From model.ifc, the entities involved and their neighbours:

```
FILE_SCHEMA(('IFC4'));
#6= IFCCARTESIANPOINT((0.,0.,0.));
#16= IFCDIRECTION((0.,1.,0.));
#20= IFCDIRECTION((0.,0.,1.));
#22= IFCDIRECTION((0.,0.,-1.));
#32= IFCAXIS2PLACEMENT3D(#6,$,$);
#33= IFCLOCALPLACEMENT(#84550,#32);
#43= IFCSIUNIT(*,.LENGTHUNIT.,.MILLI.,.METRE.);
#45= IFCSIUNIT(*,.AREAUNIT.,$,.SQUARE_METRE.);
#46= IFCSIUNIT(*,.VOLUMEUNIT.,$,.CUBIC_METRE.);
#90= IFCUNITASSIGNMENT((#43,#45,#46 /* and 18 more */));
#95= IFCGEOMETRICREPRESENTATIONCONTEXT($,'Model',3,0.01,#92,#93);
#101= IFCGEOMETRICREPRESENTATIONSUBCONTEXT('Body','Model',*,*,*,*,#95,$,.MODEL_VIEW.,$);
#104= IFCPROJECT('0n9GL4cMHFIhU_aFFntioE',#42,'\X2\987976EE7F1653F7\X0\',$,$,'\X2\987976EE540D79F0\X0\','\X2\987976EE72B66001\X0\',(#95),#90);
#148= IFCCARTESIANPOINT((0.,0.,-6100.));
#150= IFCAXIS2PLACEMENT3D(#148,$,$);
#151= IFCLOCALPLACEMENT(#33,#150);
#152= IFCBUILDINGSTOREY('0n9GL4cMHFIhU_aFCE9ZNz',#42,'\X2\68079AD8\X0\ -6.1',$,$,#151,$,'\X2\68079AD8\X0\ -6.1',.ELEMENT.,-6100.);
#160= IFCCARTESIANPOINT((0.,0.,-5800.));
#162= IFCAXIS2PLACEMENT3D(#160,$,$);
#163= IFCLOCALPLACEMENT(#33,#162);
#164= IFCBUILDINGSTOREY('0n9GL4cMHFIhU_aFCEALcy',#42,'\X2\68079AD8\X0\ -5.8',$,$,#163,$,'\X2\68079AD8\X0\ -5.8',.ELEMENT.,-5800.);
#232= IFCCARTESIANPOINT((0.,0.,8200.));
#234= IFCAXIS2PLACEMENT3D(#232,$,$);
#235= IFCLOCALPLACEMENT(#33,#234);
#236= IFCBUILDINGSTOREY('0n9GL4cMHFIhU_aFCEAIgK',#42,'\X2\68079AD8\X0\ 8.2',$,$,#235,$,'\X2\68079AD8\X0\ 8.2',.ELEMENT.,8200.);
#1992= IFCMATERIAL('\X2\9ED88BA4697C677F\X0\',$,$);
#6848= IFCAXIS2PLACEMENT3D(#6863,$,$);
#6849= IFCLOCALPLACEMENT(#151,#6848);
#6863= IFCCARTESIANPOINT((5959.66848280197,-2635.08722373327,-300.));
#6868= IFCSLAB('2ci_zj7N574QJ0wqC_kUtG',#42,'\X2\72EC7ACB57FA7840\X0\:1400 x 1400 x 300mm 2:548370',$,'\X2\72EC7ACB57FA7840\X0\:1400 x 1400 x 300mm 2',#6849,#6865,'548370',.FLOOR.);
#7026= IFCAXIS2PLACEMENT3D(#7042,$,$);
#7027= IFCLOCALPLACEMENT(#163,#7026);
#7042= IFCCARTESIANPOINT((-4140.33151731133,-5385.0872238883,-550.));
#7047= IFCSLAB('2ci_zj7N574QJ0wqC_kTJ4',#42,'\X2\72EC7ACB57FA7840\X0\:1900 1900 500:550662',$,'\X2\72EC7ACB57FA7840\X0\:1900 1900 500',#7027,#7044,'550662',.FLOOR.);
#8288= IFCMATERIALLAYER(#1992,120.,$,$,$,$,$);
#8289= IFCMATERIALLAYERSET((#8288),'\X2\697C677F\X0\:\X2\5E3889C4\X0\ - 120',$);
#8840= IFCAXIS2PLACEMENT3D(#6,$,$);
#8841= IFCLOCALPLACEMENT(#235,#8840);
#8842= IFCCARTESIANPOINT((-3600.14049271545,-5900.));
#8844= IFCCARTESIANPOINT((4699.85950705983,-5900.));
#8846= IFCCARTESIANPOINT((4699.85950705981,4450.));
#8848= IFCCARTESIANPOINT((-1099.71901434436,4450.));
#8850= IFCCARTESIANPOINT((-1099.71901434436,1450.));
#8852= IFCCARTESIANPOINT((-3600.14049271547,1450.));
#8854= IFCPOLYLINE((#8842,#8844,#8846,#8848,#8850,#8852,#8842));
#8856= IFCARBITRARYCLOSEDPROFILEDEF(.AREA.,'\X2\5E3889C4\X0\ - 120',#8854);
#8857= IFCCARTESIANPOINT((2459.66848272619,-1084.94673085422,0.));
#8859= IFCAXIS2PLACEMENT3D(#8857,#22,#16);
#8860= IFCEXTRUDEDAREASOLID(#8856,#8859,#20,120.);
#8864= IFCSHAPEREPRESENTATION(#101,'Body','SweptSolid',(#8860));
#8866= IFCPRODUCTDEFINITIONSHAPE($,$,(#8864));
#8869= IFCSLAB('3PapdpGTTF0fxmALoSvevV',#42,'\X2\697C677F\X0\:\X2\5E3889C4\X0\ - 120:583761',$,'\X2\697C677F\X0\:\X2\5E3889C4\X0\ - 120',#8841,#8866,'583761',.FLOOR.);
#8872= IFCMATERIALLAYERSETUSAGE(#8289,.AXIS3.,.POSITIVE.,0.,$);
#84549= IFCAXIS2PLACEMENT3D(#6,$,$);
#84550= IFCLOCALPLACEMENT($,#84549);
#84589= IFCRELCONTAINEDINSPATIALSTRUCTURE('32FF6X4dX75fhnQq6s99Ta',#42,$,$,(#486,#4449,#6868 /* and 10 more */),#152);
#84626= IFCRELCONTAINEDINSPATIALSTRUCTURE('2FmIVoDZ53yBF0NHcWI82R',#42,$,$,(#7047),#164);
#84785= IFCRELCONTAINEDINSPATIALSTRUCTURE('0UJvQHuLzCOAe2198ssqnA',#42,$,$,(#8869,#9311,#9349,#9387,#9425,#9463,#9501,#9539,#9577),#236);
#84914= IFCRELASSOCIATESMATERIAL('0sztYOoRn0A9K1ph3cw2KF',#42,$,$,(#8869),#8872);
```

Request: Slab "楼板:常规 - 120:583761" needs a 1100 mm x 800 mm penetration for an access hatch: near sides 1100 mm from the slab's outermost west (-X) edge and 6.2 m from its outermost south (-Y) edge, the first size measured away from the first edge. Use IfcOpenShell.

```python
import numpy as np
import ifcopenshell
import ifcopenshell.api.feature
import ifcopenshell.api.geometry
import ifcopenshell.api.root
import ifcopenshell.geom
import ifcopenshell.util.placement
import ifcopenshell.util.representation
import ifcopenshell.util.shape
import ifcopenshell.util.unit

model = ifcopenshell.open("model.ifc")
unit_scale = ifcopenshell.util.unit.calculate_unit_scale(model)
settings = ifcopenshell.geom.settings()


def volume(element):
    """Net volume in cubic metres, openings subtracted."""
    shape = ifcopenshell.geom.create_shape(settings, element)
    return ifcopenshell.util.shape.get_volume(shape.geometry)


slab = model.by_guid("3PapdpGTTF0fxmALoSvevV")
before = volume(slab)

# Extent in the slab's own axes, in metres. The edges named are its -X and -Y sides.
slab_shape = ifcopenshell.geom.create_shape(settings, slab)
vertices = ifcopenshell.util.shape.get_vertices(slab_shape.geometry)
x_min, y_min, bottom = vertices.min(axis=0)
top = vertices[:, 2].max()

opening = ifcopenshell.api.root.create_entity(model, ifc_class="IfcOpeningElement", name="Access hatch opening", predefined_type="OPENING")
context = ifcopenshell.util.representation.get_context(model, "Model", "Body", "MODEL_VIEW")
width, depth = 1.1, 0.8
outline = [(0.0, 0.0), (width, 0.0), (width, depth), (0.0, depth), (0.0, 0.0)]
# Overshoot both faces by 50 mm so the cut is clean.
shape = ifcopenshell.api.geometry.add_slab_representation(
    model, context=context, depth=top - bottom + 0.1, polyline=outline
)
ifcopenshell.api.geometry.assign_representation(model, product=opening, representation=shape)

matrix = ifcopenshell.util.placement.get_local_placement(slab.ObjectPlacement)
matrix[:, 3] = matrix @ np.append(np.array([x_min + 1.1, y_min + 6.2, bottom - 0.05]) / unit_scale, 1.0)
ifcopenshell.api.geometry.edit_object_placement(model, product=opening, matrix=matrix, is_si=False)
ifcopenshell.api.feature.add_feature(model, feature=opening, element=slab)

after = volume(slab)

print(f"slab volume {before:.3f} -> {after:.3f} m3")

model.write("model_edited.ifc")
```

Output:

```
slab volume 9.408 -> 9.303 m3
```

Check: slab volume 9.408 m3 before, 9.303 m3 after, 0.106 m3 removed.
